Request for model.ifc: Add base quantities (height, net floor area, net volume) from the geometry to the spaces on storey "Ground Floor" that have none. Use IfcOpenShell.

First a look at what the model holds.

```python
import ifcopenshell
import ifcopenshell.util.element
import ifcopenshell.util.unit

model = ifcopenshell.open("model.ifc")
print(model.schema)
for unit_type in ("LENGTHUNIT", "AREAUNIT", "VOLUMEUNIT"):
    print(unit_type, ifcopenshell.util.unit.calculate_unit_scale(model, unit_type))
storey = next(s for s in model.by_type("IfcBuildingStorey") if s.Name == "Ground Floor")
spaces = [e for e in ifcopenshell.util.element.get_decomposition(storey) if e.is_a("IfcSpace")]
for e in sorted(spaces, key=lambda e: e.id()):
    print(e.id(), e.is_a(), e.Name, list(ifcopenshell.util.element.get_psets(e, qtos_only=True)), sep=" | ")
```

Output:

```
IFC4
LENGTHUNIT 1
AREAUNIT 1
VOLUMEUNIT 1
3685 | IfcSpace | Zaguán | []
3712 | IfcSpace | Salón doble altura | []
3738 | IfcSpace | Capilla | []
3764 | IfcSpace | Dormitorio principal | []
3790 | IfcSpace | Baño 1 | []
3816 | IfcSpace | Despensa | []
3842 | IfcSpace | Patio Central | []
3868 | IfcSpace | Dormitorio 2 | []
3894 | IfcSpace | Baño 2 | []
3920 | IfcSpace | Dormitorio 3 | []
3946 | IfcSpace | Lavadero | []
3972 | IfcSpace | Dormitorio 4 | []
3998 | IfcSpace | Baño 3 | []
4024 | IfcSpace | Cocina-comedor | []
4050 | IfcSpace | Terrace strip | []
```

```python
import ifcopenshell
import ifcopenshell.api.pset
import ifcopenshell.geom
import ifcopenshell.util.element
import ifcopenshell.util.shape
import ifcopenshell.util.unit

model = ifcopenshell.open("model.ifc")
unit_scale = ifcopenshell.util.unit.calculate_unit_scale(model)
area_scale = ifcopenshell.util.unit.calculate_unit_scale(model, "AREAUNIT")
volume_scale = ifcopenshell.util.unit.calculate_unit_scale(model, "VOLUMEUNIT")
settings = ifcopenshell.geom.settings()

storey = next(s for s in model.by_type("IfcBuildingStorey") if s.Name == "Ground Floor")
spaces = [e for e in ifcopenshell.util.element.get_decomposition(storey) if e.is_a("IfcSpace")]

for e in sorted(spaces, key=lambda e: e.id()):
    if ifcopenshell.util.element.get_psets(e, qtos_only=True, should_inherit=False):
        continue
    # Geometry comes back in metres, in the element's own axes.
    shape = ifcopenshell.geom.create_shape(settings, e)
    values = {
        "Height": ifcopenshell.util.shape.get_z(shape.geometry) / unit_scale,
        "NetFloorArea": ifcopenshell.util.shape.get_footprint_area(shape.geometry) / area_scale,
        "NetVolume": ifcopenshell.util.shape.get_volume(shape.geometry) / volume_scale,
    }
    qto = ifcopenshell.api.pset.add_qto(model, product=e, name="Qto_SpaceBaseQuantities")
    ifcopenshell.api.pset.edit_qto(model, qto=qto, properties=values)
    print(e.id(), {k: round(v, 3) for k, v in values.items()})

model.write("model_edited.ifc")
```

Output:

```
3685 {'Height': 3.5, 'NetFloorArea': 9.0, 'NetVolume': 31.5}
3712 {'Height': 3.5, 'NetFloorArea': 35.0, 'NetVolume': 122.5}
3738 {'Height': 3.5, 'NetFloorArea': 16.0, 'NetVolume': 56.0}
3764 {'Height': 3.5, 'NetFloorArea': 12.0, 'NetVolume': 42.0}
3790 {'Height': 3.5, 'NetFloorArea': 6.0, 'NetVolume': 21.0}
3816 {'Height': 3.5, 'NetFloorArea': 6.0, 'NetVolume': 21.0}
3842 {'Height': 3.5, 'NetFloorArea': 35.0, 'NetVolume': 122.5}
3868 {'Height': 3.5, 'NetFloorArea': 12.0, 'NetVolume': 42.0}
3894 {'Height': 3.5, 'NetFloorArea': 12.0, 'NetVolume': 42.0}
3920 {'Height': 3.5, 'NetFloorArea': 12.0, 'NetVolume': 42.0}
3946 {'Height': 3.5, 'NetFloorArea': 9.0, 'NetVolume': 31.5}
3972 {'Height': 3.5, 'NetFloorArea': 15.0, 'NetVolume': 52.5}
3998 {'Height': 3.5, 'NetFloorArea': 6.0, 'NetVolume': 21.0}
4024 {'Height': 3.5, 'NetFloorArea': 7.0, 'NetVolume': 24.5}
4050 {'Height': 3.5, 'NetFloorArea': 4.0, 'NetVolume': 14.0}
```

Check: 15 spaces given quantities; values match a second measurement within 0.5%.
